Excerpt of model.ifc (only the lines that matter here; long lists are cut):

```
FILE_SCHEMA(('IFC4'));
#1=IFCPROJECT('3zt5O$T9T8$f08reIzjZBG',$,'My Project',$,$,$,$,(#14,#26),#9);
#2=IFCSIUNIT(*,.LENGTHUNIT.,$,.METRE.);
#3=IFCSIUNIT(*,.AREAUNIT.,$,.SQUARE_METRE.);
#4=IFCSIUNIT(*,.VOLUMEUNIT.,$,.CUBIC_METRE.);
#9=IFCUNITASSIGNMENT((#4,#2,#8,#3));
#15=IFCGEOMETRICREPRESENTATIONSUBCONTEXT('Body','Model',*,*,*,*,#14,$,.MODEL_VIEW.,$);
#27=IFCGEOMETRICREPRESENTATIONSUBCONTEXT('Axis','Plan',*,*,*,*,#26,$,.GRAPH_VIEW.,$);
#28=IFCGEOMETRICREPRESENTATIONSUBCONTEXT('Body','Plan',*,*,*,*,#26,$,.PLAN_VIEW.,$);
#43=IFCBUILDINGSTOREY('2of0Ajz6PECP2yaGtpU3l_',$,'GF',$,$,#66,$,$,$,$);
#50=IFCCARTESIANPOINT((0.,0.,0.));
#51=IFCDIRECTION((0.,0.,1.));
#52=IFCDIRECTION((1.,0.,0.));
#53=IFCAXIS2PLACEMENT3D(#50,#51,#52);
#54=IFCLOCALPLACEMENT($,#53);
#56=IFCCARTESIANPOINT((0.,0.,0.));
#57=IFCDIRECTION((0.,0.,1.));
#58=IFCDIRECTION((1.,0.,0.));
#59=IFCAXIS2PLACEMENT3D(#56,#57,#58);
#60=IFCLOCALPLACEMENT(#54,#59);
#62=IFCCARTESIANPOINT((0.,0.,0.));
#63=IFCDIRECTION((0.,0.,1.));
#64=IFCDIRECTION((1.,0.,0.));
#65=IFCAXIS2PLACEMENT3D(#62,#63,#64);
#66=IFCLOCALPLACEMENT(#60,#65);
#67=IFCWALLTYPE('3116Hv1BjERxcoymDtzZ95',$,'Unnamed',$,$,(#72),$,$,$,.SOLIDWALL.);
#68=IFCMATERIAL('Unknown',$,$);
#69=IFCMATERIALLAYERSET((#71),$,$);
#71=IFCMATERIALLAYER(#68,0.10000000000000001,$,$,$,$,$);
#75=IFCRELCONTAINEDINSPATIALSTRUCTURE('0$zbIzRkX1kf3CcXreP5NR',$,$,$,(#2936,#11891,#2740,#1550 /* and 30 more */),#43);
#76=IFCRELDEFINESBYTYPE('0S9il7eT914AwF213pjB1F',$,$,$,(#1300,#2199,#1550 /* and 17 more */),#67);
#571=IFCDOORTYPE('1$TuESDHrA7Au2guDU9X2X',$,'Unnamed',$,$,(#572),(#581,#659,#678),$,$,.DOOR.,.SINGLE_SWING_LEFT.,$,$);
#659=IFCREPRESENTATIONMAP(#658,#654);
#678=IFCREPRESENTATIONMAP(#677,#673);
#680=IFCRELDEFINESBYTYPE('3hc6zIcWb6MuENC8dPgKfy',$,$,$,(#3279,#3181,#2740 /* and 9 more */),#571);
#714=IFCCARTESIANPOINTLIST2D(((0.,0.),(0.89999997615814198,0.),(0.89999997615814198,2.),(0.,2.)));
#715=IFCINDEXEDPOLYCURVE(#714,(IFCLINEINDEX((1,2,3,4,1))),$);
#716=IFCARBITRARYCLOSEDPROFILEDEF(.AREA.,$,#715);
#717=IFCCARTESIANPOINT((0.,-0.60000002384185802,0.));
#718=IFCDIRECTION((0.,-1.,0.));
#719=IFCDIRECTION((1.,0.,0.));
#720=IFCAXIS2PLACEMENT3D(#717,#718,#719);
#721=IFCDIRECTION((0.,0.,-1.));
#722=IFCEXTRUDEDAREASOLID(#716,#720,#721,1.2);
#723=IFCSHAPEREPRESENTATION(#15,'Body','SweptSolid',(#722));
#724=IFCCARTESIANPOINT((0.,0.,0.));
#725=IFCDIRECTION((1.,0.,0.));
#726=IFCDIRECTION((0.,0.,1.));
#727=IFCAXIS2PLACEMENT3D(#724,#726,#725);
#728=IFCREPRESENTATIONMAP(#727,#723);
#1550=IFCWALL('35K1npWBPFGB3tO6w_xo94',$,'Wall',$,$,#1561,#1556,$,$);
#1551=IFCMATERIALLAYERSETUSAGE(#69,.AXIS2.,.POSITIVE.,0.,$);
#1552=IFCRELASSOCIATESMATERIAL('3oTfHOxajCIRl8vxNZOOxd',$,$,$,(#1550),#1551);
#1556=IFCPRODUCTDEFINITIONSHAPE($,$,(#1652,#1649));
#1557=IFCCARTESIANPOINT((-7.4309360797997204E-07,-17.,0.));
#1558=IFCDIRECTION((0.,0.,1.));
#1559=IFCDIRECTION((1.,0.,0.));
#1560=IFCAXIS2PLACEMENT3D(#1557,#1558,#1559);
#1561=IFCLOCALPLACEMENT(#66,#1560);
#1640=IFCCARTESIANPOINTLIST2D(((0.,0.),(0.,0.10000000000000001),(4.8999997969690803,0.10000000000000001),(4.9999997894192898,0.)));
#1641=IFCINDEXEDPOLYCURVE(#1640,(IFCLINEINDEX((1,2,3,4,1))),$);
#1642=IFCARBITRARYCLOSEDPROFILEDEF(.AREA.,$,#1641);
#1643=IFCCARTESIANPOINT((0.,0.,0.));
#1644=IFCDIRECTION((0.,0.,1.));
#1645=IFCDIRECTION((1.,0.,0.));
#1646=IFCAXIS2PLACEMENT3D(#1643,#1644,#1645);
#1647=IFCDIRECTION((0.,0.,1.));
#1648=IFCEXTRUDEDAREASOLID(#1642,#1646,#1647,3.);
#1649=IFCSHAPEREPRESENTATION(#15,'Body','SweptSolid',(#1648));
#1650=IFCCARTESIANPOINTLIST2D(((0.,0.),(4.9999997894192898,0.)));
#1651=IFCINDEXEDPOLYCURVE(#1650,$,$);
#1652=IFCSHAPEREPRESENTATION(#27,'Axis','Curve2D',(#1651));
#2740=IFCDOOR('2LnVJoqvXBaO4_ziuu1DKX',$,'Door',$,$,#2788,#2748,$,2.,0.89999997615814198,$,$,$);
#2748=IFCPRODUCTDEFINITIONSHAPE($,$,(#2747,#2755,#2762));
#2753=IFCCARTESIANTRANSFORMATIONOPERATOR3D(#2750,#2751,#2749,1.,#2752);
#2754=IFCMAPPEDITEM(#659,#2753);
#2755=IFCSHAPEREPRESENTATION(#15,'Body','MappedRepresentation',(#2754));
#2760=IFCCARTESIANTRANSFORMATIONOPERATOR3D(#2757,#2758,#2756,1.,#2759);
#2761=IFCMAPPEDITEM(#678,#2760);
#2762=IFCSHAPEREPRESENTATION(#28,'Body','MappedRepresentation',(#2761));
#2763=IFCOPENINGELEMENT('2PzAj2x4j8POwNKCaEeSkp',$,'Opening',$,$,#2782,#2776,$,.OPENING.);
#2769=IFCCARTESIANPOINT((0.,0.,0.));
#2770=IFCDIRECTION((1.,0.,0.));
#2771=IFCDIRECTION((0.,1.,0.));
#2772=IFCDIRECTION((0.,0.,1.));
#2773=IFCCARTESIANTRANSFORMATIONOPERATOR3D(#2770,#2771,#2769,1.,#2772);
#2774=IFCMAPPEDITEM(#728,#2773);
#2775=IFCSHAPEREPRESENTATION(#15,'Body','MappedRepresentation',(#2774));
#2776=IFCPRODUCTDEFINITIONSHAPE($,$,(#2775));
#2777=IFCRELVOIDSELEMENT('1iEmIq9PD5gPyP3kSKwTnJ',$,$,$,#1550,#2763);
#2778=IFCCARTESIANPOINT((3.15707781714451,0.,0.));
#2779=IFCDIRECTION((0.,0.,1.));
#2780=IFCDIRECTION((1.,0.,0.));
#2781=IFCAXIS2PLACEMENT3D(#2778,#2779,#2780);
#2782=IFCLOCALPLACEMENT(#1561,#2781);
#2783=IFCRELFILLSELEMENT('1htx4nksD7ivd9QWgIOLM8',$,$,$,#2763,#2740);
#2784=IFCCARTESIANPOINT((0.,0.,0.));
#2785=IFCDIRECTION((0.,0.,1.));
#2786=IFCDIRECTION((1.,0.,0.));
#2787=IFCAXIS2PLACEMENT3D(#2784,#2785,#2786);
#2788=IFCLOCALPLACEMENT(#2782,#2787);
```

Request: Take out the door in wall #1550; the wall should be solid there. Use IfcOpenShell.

```python
import ifcopenshell
import ifcopenshell.api.feature
import ifcopenshell.api.root
import ifcopenshell.geom
import ifcopenshell.util.shape

model = ifcopenshell.open("model.ifc")
settings = ifcopenshell.geom.settings()


def volume(element):
    """Net volume in cubic metres, openings subtracted."""
    shape = ifcopenshell.geom.create_shape(settings, element)
    return ifcopenshell.util.shape.get_volume(shape.geometry)


door = model.by_guid("2LnVJoqvXBaO4_ziuu1DKX")
opening = door.FillsVoids[0].RelatingOpeningElement
wall = opening.VoidsElements[0].RelatingBuildingElement
before = volume(wall)

ifcopenshell.api.root.remove_product(model, product=door)
ifcopenshell.api.feature.remove_feature(model, feature=opening)

after = volume(wall)

print(f"wall volume {before:.3f} -> {after:.3f} m3")

model.write("model_rev.ifc")
```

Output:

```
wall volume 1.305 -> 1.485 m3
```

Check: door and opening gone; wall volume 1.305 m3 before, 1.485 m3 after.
